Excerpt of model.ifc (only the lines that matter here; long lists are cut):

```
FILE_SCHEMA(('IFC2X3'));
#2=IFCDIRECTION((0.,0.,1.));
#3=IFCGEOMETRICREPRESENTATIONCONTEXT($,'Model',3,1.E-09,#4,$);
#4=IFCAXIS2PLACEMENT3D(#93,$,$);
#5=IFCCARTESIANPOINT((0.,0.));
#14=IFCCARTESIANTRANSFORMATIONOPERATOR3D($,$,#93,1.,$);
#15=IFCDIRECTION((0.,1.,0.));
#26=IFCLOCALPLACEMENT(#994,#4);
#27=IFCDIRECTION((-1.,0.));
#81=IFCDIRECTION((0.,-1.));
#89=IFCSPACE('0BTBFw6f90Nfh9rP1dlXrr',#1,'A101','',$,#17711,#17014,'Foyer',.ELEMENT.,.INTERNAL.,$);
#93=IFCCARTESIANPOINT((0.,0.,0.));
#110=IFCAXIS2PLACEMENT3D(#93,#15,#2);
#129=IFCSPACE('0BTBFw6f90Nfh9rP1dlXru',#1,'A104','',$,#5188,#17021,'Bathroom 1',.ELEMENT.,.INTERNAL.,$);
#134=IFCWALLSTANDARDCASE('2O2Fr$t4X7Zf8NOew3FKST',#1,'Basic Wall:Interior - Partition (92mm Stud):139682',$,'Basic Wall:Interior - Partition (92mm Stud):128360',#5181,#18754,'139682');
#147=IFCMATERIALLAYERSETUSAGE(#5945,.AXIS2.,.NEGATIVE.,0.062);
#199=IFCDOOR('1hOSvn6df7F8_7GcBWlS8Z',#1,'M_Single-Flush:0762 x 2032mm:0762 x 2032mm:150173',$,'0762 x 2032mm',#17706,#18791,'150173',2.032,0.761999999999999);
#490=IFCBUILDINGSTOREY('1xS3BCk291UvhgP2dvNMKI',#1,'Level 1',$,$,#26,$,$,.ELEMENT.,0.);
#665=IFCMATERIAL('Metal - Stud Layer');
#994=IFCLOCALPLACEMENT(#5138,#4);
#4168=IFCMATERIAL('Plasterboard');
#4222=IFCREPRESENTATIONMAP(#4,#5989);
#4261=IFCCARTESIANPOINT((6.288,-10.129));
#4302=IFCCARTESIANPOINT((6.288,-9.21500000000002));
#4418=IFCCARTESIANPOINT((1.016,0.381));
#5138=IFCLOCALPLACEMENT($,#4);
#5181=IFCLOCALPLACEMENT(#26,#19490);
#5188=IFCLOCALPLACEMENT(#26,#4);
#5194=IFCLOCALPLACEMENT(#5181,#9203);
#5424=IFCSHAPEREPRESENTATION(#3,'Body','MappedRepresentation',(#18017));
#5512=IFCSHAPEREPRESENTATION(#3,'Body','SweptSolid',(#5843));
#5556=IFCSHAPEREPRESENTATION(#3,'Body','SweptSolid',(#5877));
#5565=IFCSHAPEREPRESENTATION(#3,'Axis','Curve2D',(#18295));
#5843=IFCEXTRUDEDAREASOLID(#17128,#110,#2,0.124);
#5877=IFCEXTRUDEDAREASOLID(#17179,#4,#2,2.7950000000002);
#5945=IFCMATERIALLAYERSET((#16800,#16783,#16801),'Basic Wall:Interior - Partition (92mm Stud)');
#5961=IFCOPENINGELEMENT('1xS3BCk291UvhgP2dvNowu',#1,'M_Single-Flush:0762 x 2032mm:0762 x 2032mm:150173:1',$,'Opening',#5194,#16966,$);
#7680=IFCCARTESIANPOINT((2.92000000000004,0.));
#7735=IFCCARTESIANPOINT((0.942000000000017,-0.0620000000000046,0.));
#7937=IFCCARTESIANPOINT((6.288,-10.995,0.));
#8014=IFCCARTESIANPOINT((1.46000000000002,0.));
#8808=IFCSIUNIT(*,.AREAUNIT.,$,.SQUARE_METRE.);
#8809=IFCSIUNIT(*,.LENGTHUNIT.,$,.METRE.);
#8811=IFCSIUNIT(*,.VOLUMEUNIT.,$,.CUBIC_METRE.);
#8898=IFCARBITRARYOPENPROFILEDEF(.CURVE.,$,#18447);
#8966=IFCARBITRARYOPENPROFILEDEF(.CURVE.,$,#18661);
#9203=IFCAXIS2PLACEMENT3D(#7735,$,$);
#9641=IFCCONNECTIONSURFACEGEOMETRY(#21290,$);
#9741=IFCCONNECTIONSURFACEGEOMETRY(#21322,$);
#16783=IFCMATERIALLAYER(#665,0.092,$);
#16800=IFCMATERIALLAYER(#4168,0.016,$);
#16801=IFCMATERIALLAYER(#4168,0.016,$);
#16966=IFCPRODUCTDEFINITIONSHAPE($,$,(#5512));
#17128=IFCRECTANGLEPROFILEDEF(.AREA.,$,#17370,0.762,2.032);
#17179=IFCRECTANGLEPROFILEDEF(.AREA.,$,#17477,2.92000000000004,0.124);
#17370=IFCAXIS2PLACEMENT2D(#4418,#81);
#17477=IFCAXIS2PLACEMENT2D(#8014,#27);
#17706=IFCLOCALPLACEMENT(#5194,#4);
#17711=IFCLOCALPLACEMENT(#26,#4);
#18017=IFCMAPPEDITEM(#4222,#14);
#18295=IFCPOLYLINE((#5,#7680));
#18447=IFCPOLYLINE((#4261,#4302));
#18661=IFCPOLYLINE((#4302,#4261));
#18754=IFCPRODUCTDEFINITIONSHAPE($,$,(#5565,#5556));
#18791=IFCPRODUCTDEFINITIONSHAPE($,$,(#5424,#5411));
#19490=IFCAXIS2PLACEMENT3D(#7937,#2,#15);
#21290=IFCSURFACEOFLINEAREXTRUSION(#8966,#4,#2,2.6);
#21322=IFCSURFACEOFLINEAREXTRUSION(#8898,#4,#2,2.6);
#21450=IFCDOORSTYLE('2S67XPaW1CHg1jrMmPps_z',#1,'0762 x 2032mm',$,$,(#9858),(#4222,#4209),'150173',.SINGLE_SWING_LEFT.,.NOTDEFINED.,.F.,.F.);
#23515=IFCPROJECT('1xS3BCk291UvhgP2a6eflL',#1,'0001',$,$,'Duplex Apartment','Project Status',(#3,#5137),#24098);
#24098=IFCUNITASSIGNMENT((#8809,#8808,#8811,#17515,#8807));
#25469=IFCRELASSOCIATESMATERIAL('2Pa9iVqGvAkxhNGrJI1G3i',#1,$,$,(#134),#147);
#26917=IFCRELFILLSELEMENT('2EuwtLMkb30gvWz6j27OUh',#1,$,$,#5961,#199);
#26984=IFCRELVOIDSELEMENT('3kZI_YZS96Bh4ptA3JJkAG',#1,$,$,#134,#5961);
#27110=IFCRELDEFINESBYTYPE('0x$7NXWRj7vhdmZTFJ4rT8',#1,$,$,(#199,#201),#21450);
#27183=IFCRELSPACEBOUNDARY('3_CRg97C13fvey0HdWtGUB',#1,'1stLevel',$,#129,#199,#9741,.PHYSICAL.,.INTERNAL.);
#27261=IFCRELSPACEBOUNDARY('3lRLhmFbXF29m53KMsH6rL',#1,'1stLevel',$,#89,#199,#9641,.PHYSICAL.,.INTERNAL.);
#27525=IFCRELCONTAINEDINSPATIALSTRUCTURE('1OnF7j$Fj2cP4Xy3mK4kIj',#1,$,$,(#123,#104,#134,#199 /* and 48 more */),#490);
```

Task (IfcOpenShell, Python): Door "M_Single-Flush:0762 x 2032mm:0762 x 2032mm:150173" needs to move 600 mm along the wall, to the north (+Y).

```python
import numpy as np
import ifcopenshell
import ifcopenshell.api.geometry
import ifcopenshell.util.placement

model = ifcopenshell.open("model.ifc")

door = model.by_guid("1hOSvn6df7F8_7GcBWlS8Z")
opening = door.FillsVoids[0].RelatingOpeningElement
wall = opening.VoidsElements[0].RelatingBuildingElement

wall_matrix = ifcopenshell.util.placement.get_local_placement(wall.ObjectPlacement)
shift = wall_matrix[:3, 0] * 0.6
before = ifcopenshell.util.placement.get_local_placement(door.ObjectPlacement)[:3, 3].copy()

# The door is placed relative to its opening, so it follows when the opening moves.
matrix = ifcopenshell.util.placement.get_local_placement(opening.ObjectPlacement)
matrix[:3, 3] += shift
ifcopenshell.api.geometry.edit_object_placement(
    model, product=opening, matrix=matrix, is_si=False, should_transform_children=True
)

# Space boundary surfaces are stored in each space's coordinates; move them too.
for rel in door.ProvidesBoundaries:
    if not rel.ConnectionGeometry:
        continue
    surface = rel.ConnectionGeometry.SurfaceOnRelatingElement
    space_matrix = ifcopenshell.util.placement.get_local_placement(rel.RelatingSpace.ObjectPlacement)
    point = np.array(surface.Position.Location.Coordinates) + space_matrix[:3, :3].T @ shift
    surface.Position = model.createIfcAxis2Placement3D(
        model.createIfcCartesianPoint(point.tolist()), surface.Position.Axis, surface.Position.RefDirection
    )

after = ifcopenshell.util.placement.get_local_placement(door.ObjectPlacement)[:3, 3]
print("door moved by", (after - before).round(3) + 0.0)

model.write("model-out.ifc")
```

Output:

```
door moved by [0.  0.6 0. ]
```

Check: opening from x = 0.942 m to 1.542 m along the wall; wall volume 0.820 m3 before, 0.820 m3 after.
